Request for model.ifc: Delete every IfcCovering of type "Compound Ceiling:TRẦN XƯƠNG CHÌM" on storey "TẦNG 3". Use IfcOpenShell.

First a look at what the model holds.

```python
import ifcopenshell
import ifcopenshell.util.element

model = ifcopenshell.open("model.ifc")
print(model.schema)
storey = next(s for s in model.by_type("IfcBuildingStorey") if s.Name == "TẦNG 3")
coverings = [e for e in ifcopenshell.util.element.get_decomposition(storey) if e.is_a("IfcCovering")]
seen = {}
for e in coverings:
    element_type = ifcopenshell.util.element.get_type(e)
    name = element_type.Name if element_type not in (None, e) else None
    seen[name] = seen.get(name, 0) + 1
for name, count in sorted(seen.items(), key=str):
    print(count, "x", name)
```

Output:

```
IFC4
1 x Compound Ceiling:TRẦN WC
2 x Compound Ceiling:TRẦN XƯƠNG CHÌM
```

```python
import ifcopenshell
import ifcopenshell.api.root
import ifcopenshell.util.element

model = ifcopenshell.open("model.ifc")

storey = next(s for s in model.by_type("IfcBuildingStorey") if s.Name == "TẦNG 3")
coverings = [e for e in ifcopenshell.util.element.get_decomposition(storey) if e.is_a("IfcCovering")]
targets = [e for e in coverings if (t := ifcopenshell.util.element.get_type(e)) not in (None, e) and t.Name == "Compound Ceiling:TRẦN XƯƠNG CHÌM"]

for e in targets:
    ifcopenshell.api.root.remove_product(model, product=e)
print(len(targets), "removed")

model.write("model-out.ifc")
```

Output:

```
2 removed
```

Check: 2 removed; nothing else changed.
